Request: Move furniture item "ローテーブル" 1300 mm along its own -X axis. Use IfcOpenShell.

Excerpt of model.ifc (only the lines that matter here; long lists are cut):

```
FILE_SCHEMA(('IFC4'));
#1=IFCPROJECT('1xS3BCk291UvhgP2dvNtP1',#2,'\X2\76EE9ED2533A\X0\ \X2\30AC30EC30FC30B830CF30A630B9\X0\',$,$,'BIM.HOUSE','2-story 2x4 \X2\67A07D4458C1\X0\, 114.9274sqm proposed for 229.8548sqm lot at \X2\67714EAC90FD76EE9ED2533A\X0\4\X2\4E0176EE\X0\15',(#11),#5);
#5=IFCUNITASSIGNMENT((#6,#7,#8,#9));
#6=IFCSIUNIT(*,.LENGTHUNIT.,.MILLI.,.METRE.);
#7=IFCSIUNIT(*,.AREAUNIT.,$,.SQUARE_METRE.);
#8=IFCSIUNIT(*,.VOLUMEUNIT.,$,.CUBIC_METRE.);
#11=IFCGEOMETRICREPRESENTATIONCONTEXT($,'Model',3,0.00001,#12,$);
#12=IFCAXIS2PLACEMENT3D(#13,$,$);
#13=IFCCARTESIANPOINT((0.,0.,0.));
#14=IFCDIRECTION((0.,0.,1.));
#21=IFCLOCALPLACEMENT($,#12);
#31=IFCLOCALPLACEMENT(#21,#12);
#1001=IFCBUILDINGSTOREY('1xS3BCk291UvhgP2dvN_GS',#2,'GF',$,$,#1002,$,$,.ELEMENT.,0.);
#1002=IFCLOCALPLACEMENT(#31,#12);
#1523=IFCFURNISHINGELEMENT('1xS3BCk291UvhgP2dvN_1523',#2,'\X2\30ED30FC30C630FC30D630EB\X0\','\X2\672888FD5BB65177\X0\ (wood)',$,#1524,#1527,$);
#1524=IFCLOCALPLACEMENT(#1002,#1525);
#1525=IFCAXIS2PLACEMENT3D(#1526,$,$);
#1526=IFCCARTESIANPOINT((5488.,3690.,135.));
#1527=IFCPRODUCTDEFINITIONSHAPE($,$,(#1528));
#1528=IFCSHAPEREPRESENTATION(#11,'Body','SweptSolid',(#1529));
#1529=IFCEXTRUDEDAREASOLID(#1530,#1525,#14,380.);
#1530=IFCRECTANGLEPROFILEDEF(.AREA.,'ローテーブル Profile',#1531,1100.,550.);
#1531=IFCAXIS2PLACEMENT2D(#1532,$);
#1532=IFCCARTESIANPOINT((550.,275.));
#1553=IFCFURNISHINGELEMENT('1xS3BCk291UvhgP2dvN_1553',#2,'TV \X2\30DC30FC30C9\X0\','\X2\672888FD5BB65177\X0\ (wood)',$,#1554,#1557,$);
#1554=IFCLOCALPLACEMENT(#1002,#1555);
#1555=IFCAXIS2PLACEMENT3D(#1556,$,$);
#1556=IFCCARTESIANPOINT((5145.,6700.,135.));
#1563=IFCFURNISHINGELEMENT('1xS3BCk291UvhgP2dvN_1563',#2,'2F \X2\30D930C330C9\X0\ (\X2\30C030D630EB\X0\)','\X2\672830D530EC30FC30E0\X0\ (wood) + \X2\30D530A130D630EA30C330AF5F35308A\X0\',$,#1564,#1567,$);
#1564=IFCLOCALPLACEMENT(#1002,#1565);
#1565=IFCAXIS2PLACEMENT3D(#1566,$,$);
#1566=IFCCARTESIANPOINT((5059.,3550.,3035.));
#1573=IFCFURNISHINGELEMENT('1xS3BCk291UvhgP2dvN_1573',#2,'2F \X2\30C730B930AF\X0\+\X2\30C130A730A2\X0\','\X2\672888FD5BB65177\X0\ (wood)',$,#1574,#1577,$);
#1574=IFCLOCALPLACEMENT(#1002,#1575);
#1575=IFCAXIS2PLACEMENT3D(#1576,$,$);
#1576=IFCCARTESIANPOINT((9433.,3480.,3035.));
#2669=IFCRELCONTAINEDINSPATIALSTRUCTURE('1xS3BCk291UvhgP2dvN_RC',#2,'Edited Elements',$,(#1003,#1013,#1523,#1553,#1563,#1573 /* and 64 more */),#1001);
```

```python
import ifcopenshell
import ifcopenshell.api.geometry
import ifcopenshell.util.placement
import ifcopenshell.util.unit

model = ifcopenshell.open("model.ifc")
unit_scale = ifcopenshell.util.unit.calculate_unit_scale(model)

item = model.by_guid("1xS3BCk291UvhgP2dvN_1523")
matrix = ifcopenshell.util.placement.get_local_placement(item.ObjectPlacement)
matrix[:3, 3] -= matrix[:3, 0] * 1.3 / unit_scale
ifcopenshell.api.geometry.edit_object_placement(model, product=item, matrix=matrix, is_si=False)

print(ifcopenshell.util.placement.get_local_placement(item.ObjectPlacement).round(3) + 0.0)

model.write("model-out.ifc")
```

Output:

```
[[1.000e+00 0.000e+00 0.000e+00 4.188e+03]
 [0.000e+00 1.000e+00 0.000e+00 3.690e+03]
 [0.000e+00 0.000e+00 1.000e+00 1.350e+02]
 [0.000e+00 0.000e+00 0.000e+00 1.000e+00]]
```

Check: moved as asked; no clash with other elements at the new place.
